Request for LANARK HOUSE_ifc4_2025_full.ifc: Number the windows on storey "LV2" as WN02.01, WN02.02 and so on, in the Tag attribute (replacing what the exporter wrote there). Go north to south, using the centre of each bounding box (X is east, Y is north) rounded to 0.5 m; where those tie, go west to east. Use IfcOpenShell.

First a look at what the model holds.

```python
import ifcopenshell
import ifcopenshell.util.element
import ifcopenshell.util.placement

model = ifcopenshell.open("LANARK HOUSE_ifc4_2025_full.ifc")
print(model.schema)
storey = next(s for s in model.by_type("IfcBuildingStorey") if s.Name == "LV2")
windows = [e for e in ifcopenshell.util.element.get_decomposition(storey) if e.is_a("IfcWindow")]
for e in sorted(windows, key=lambda e: e.id()):
    origin = ifcopenshell.util.placement.get_local_placement(e.ObjectPlacement)[:3, 3]
    print(e.id(), e.Tag, e.Name, origin.round(2) + 0.0, sep=" | ")
```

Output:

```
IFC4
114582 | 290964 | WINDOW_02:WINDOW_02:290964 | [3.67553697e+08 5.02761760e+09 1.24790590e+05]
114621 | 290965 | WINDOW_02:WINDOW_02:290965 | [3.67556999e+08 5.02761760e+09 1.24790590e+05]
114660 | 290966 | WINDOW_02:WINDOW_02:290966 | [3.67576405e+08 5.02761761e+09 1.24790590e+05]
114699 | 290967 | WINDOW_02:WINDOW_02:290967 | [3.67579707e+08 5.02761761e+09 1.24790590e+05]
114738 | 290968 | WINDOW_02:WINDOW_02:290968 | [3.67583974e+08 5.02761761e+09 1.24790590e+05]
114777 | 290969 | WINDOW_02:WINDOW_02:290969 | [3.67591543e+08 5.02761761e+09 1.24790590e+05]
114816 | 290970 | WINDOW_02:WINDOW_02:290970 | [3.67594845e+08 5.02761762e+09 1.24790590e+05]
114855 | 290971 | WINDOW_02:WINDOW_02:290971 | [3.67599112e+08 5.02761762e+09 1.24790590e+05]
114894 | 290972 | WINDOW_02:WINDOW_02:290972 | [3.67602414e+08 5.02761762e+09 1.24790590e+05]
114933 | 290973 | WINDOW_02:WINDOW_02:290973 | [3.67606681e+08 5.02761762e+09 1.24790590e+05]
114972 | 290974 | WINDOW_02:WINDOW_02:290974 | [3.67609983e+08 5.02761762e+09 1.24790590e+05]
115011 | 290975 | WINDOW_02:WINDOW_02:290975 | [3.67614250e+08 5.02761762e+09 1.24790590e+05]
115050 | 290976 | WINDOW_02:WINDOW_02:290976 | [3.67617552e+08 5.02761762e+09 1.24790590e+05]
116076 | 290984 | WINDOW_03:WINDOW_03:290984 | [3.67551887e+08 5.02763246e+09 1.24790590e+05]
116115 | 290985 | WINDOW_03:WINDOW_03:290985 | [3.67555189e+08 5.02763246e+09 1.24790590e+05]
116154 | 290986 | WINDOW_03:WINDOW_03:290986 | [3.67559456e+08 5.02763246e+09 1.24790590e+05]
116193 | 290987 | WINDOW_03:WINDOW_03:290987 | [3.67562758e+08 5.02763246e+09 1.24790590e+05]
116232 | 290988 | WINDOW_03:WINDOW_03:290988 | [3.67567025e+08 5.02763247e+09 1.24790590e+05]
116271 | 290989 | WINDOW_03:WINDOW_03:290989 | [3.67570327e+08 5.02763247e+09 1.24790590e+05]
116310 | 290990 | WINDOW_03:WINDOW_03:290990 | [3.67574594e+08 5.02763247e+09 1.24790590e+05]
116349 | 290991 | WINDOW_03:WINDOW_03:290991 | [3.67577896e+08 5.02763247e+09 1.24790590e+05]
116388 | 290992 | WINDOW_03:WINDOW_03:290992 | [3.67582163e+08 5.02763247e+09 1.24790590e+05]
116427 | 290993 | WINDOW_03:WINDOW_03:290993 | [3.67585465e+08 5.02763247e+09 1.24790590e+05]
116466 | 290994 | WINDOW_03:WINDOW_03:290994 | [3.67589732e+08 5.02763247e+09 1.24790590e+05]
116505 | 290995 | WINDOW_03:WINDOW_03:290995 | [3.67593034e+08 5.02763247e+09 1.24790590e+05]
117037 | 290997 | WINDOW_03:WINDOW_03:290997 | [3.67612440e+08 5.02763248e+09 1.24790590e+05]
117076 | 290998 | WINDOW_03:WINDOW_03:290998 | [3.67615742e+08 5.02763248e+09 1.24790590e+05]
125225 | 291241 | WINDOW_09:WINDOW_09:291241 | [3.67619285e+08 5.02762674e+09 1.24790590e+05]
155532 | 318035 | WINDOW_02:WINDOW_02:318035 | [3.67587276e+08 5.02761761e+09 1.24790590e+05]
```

```python
import ifcopenshell
import ifcopenshell.geom
import ifcopenshell.util.element
import ifcopenshell.util.shape

model = ifcopenshell.open("LANARK HOUSE_ifc4_2025_full.ifc")
settings = ifcopenshell.geom.settings()
settings.set("use-world-coords", True)


def centre(element):
    shape = ifcopenshell.geom.create_shape(settings, element)
    return ifcopenshell.util.shape.get_bbox_centroid(shape.geometry)


storey = next(s for s in model.by_type("IfcBuildingStorey") if s.Name == "LV2")
windows = [e for e in ifcopenshell.util.element.get_decomposition(storey) if e.is_a("IfcWindow")]

# Insertion points can sit at a corner or the storey origin, so sort by the geometry (in metres).
centres = {e: centre(e) for e in windows}
windows.sort(key=lambda e: (-round(centres[e][1] / 0.5), centres[e][0]))

for i, e in enumerate(windows, start=1):
    number = f"WN02.{i:02d}"
    e.Tag = number
    print(e.id(), number)

model.write("LANARK HOUSE_ifc4_2025_full_edited.ifc")
```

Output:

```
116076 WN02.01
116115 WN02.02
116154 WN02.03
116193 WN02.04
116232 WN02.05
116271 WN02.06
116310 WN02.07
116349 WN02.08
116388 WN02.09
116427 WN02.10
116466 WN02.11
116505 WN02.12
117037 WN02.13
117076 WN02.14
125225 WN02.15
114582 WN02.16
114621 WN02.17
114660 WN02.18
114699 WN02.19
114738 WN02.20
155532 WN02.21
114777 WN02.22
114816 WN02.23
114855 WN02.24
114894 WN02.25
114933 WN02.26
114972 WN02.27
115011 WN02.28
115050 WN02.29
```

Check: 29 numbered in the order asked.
